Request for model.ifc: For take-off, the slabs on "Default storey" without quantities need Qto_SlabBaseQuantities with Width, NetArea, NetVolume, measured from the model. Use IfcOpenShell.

First a look at what the model holds.

```python
import ifcopenshell
import ifcopenshell.util.element
import ifcopenshell.util.unit

model = ifcopenshell.open("model.ifc")
print(model.schema)
for unit_type in ("LENGTHUNIT", "AREAUNIT", "VOLUMEUNIT"):
    print(unit_type, ifcopenshell.util.unit.calculate_unit_scale(model, unit_type))
storey = next(s for s in model.by_type("IfcBuildingStorey") if s.Name == "Default storey")
slabs = [e for e in ifcopenshell.util.element.get_decomposition(storey) if e.is_a("IfcSlab")]
for e in sorted(slabs, key=lambda e: e.id()):
    print(e.id(), e.is_a(), e.Name, list(ifcopenshell.util.element.get_psets(e, qtos_only=True)), sep=" | ")
```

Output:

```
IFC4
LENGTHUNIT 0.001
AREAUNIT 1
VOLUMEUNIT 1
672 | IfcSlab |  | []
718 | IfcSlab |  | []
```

```python
import ifcopenshell
import ifcopenshell.api.pset
import ifcopenshell.geom
import ifcopenshell.util.element
import ifcopenshell.util.shape
import ifcopenshell.util.unit

model = ifcopenshell.open("model.ifc")
unit_scale = ifcopenshell.util.unit.calculate_unit_scale(model)
area_scale = ifcopenshell.util.unit.calculate_unit_scale(model, "AREAUNIT")
volume_scale = ifcopenshell.util.unit.calculate_unit_scale(model, "VOLUMEUNIT")
settings = ifcopenshell.geom.settings()

storey = next(s for s in model.by_type("IfcBuildingStorey") if s.Name == "Default storey")
slabs = [e for e in ifcopenshell.util.element.get_decomposition(storey) if e.is_a("IfcSlab")]

for e in sorted(slabs, key=lambda e: e.id()):
    if ifcopenshell.util.element.get_psets(e, qtos_only=True, should_inherit=False):
        continue
    # Geometry comes back in metres, in the element's own axes.
    shape = ifcopenshell.geom.create_shape(settings, e)
    values = {
        "Width": ifcopenshell.util.shape.get_z(shape.geometry) / unit_scale,
        "NetArea": ifcopenshell.util.shape.get_footprint_area(shape.geometry) / area_scale,
        "NetVolume": ifcopenshell.util.shape.get_volume(shape.geometry) / volume_scale,
    }
    qto = ifcopenshell.api.pset.add_qto(model, product=e, name="Qto_SlabBaseQuantities")
    ifcopenshell.api.pset.edit_qto(model, qto=qto, properties=values)
    print(e.id(), {k: round(v, 3) for k, v in values.items()})

model.write("model_v2.ifc")
```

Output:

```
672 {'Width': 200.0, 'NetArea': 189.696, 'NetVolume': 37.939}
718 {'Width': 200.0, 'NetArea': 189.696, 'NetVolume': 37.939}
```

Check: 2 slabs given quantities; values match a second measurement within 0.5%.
